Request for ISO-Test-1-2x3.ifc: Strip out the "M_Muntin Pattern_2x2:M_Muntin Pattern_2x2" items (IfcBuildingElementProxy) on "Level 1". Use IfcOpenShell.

First a look at what the model holds.

```python
import ifcopenshell
import ifcopenshell.util.element

model = ifcopenshell.open("ISO-Test-1-2x3.ifc")
print(model.schema)
storey = next(s for s in model.by_type("IfcBuildingStorey") if s.Name == "Level 1")
proxies = [e for e in ifcopenshell.util.element.get_decomposition(storey) if e.is_a("IfcBuildingElementProxy")]
seen = {}
for e in proxies:
    element_type = ifcopenshell.util.element.get_type(e)
    name = element_type.Name if element_type not in (None, e) else None
    seen[name] = seen.get(name, 0) + 1
for name, count in sorted(seen.items(), key=str):
    print(count, "x", name)
```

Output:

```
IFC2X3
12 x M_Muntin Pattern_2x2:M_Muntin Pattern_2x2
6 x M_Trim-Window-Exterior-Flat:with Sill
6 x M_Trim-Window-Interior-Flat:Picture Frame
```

```python
import ifcopenshell
import ifcopenshell.api.root
import ifcopenshell.util.element

model = ifcopenshell.open("ISO-Test-1-2x3.ifc")

storey = next(s for s in model.by_type("IfcBuildingStorey") if s.Name == "Level 1")
proxies = [e for e in ifcopenshell.util.element.get_decomposition(storey) if e.is_a("IfcBuildingElementProxy")]
targets = [e for e in proxies if (t := ifcopenshell.util.element.get_type(e)) not in (None, e) and t.Name == "M_Muntin Pattern_2x2:M_Muntin Pattern_2x2"]

for e in targets:
    ifcopenshell.api.root.remove_product(model, product=e)
print(len(targets), "removed")

model.write("ISO-Test-1-2x3_v2.ifc")
```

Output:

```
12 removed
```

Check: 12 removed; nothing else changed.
